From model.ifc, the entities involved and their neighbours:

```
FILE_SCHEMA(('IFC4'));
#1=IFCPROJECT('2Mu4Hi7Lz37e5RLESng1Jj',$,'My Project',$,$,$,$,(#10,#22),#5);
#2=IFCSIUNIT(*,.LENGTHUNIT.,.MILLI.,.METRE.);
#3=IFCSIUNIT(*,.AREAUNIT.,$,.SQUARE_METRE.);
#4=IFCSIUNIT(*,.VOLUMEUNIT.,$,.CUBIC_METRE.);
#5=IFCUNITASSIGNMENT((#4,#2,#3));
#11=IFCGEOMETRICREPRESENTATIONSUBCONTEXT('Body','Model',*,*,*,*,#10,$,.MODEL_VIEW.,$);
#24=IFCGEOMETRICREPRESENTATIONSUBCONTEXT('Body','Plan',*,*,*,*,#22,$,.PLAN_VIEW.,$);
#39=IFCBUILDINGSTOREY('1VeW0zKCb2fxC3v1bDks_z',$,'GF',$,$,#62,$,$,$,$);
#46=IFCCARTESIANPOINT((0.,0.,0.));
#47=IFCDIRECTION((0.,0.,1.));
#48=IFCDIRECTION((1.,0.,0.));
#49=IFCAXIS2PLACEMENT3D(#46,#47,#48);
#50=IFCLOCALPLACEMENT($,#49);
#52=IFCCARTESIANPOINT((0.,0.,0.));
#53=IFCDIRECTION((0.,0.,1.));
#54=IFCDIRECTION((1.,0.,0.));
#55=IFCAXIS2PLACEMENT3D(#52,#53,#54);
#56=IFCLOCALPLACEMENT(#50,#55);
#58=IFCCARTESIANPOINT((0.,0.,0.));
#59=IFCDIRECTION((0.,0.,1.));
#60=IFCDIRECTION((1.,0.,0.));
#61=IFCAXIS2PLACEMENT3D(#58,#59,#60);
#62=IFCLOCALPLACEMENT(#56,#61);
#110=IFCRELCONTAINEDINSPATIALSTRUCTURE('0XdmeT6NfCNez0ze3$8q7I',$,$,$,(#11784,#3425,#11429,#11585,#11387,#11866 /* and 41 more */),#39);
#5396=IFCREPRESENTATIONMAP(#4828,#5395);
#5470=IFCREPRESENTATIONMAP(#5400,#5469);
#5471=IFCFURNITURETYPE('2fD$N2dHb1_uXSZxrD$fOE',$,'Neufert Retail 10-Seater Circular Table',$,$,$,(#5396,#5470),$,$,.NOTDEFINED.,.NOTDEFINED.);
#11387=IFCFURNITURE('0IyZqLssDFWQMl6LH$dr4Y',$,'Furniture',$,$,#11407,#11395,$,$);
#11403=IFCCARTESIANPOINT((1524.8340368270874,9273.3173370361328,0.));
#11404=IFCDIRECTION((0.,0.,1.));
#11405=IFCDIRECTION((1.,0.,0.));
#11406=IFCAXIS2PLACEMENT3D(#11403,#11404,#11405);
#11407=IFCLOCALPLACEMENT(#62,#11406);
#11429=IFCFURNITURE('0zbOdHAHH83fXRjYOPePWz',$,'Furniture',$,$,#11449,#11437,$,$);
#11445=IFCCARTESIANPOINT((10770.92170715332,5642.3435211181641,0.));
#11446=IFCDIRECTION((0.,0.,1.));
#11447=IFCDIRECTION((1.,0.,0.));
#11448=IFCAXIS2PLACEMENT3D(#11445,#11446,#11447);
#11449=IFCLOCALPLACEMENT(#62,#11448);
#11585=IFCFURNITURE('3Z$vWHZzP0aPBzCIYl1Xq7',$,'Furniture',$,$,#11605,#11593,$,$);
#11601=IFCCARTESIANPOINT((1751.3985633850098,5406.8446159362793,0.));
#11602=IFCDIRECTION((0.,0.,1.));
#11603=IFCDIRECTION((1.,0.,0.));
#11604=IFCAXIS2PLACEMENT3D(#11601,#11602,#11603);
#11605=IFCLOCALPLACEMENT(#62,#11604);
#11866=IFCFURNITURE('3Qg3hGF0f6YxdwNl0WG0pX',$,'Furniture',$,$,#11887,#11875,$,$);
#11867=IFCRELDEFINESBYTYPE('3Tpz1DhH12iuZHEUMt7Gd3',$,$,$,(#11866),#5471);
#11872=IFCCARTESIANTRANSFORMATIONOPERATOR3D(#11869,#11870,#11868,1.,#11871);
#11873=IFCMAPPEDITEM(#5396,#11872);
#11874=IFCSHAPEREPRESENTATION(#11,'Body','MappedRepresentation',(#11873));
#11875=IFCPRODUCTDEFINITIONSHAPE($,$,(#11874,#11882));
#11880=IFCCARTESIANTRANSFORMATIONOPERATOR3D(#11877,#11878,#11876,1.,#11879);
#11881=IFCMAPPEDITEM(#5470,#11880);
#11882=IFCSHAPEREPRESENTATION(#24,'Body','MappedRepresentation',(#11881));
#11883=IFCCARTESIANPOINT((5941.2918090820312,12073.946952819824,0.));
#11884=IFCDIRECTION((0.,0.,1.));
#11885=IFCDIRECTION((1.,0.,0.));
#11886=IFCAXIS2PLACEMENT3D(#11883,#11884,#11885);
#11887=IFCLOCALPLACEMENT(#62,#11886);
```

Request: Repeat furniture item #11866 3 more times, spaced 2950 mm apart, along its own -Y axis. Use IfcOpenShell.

```python
import ifcopenshell
import ifcopenshell.api.geometry
import ifcopenshell.api.root
import ifcopenshell.util.element
import ifcopenshell.util.placement

model = ifcopenshell.open("model.ifc")

source = model.by_guid("3Qg3hGF0f6YxdwNl0WG0pX")
base = ifcopenshell.util.placement.get_local_placement(source.ObjectPlacement)
step = -base[:3, 1] * 2950.0

for i in range(1, 4):
    copy = ifcopenshell.api.root.copy_class(model, product=source)
    copy.Representation = ifcopenshell.util.element.copy_deep(
        model, source.Representation, exclude=["IfcGeometricRepresentationContext", "IfcRepresentationMap"]
    )
    matrix = base.copy()
    matrix[:3, 3] += i * step
    print("added at", matrix[:3, 3].round(3) + 0.0)
    ifcopenshell.api.geometry.edit_object_placement(model, product=copy, matrix=matrix, is_si=False)

model.write("model_updated.ifc")
```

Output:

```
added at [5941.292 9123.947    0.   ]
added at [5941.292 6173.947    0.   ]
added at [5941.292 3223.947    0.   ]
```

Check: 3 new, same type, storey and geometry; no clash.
